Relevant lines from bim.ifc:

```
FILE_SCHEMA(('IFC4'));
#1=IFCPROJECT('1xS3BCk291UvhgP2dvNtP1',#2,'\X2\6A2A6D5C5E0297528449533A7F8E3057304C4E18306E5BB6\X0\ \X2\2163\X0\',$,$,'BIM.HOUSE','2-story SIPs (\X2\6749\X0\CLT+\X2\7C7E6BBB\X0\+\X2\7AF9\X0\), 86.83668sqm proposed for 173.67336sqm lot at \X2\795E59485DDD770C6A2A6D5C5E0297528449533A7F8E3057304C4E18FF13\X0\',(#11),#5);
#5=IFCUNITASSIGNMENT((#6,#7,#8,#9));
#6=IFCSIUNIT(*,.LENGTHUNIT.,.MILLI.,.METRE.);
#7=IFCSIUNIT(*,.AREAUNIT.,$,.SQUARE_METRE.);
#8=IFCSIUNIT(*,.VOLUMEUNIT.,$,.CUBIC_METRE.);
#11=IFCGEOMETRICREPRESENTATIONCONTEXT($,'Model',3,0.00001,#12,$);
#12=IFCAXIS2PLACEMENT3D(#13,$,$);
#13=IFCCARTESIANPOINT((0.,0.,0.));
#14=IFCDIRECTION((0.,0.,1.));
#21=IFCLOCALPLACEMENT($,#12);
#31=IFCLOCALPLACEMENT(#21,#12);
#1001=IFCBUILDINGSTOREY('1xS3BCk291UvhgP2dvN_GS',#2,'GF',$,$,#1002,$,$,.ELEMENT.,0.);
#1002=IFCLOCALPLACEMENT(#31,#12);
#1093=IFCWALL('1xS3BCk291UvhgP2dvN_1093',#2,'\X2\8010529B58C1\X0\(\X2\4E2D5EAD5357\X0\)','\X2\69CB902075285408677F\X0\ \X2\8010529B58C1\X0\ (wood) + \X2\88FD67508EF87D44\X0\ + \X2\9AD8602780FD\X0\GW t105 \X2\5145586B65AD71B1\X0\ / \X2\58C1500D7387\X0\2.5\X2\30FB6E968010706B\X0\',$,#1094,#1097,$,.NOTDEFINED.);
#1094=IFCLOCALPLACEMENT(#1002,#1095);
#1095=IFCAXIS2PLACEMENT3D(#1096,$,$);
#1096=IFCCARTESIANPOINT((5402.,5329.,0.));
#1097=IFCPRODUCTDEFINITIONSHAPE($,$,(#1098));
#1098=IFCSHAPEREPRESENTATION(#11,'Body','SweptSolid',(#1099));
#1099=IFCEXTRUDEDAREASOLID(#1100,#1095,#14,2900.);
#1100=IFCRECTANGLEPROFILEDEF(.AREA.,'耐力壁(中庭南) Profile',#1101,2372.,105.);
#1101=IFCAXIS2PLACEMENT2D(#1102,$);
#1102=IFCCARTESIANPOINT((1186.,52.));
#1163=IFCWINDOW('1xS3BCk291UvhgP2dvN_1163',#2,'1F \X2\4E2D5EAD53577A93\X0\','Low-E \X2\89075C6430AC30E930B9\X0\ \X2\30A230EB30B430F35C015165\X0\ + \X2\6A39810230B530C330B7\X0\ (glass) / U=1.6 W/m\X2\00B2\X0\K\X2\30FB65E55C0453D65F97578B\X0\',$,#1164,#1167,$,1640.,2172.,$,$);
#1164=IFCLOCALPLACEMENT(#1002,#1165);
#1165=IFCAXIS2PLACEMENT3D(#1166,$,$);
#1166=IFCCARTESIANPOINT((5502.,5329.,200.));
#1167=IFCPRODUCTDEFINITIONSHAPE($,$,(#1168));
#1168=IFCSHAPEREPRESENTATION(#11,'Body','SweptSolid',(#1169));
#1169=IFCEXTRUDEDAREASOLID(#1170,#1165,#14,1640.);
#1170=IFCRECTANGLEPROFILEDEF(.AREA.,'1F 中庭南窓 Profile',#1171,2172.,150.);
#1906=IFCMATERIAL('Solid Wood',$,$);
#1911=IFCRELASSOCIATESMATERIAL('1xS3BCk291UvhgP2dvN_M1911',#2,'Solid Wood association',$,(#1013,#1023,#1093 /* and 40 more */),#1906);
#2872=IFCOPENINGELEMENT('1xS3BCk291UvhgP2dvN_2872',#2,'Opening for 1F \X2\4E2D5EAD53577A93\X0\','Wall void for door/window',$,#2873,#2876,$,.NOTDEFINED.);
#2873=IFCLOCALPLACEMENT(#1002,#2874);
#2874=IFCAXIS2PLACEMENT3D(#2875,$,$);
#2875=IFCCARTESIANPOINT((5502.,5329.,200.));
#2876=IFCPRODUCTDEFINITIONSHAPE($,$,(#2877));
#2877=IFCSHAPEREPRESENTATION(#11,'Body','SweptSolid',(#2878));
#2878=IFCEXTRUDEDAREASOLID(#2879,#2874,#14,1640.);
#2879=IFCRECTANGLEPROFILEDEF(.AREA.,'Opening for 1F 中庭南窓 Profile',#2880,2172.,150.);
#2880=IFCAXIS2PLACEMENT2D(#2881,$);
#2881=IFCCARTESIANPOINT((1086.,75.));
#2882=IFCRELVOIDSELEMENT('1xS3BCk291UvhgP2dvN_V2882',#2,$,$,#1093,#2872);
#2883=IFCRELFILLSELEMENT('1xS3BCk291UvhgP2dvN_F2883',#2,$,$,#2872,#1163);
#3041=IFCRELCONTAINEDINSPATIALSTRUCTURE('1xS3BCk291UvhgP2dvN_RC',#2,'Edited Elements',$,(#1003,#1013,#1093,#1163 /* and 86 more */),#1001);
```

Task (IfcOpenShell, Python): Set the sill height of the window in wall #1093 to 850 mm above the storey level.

```python
import numpy as np
import ifcopenshell
import ifcopenshell.api.geometry
import ifcopenshell.geom
import ifcopenshell.util.element
import ifcopenshell.util.placement
import ifcopenshell.util.shape
import ifcopenshell.util.unit

model = ifcopenshell.open("bim.ifc")
unit_scale = ifcopenshell.util.unit.calculate_unit_scale(model)

window = model.by_guid("1xS3BCk291UvhgP2dvN_1163")
opening = window.FillsVoids[0].RelatingOpeningElement
storey = ifcopenshell.util.element.get_container(window, ifc_class="IfcBuildingStorey")
level = ifcopenshell.util.placement.get_local_placement(storey.ObjectPlacement)[2, 3]

# The opening's origin need not be at the sill, so measure its lowest point.
shape = ifcopenshell.geom.create_shape(ifcopenshell.geom.settings(), opening)
bottom = ifcopenshell.util.shape.get_shape_bottom_elevation(shape, shape.geometry) / unit_scale
dz = level + 850.0 - bottom

shift = np.array([0.0, 0.0, dz])
# The window is not placed relative to its opening, so move both.
for product in (opening, window):
    matrix = ifcopenshell.util.placement.get_local_placement(product.ObjectPlacement)
    matrix[:3, 3] += shift
    ifcopenshell.api.geometry.edit_object_placement(model, product=product, matrix=matrix, is_si=False)

print(f"moved by {dz * unit_scale:+.3f} m")

model.write("bim_rev.ifc")
```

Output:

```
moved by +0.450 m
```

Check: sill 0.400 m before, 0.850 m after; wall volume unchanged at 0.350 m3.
